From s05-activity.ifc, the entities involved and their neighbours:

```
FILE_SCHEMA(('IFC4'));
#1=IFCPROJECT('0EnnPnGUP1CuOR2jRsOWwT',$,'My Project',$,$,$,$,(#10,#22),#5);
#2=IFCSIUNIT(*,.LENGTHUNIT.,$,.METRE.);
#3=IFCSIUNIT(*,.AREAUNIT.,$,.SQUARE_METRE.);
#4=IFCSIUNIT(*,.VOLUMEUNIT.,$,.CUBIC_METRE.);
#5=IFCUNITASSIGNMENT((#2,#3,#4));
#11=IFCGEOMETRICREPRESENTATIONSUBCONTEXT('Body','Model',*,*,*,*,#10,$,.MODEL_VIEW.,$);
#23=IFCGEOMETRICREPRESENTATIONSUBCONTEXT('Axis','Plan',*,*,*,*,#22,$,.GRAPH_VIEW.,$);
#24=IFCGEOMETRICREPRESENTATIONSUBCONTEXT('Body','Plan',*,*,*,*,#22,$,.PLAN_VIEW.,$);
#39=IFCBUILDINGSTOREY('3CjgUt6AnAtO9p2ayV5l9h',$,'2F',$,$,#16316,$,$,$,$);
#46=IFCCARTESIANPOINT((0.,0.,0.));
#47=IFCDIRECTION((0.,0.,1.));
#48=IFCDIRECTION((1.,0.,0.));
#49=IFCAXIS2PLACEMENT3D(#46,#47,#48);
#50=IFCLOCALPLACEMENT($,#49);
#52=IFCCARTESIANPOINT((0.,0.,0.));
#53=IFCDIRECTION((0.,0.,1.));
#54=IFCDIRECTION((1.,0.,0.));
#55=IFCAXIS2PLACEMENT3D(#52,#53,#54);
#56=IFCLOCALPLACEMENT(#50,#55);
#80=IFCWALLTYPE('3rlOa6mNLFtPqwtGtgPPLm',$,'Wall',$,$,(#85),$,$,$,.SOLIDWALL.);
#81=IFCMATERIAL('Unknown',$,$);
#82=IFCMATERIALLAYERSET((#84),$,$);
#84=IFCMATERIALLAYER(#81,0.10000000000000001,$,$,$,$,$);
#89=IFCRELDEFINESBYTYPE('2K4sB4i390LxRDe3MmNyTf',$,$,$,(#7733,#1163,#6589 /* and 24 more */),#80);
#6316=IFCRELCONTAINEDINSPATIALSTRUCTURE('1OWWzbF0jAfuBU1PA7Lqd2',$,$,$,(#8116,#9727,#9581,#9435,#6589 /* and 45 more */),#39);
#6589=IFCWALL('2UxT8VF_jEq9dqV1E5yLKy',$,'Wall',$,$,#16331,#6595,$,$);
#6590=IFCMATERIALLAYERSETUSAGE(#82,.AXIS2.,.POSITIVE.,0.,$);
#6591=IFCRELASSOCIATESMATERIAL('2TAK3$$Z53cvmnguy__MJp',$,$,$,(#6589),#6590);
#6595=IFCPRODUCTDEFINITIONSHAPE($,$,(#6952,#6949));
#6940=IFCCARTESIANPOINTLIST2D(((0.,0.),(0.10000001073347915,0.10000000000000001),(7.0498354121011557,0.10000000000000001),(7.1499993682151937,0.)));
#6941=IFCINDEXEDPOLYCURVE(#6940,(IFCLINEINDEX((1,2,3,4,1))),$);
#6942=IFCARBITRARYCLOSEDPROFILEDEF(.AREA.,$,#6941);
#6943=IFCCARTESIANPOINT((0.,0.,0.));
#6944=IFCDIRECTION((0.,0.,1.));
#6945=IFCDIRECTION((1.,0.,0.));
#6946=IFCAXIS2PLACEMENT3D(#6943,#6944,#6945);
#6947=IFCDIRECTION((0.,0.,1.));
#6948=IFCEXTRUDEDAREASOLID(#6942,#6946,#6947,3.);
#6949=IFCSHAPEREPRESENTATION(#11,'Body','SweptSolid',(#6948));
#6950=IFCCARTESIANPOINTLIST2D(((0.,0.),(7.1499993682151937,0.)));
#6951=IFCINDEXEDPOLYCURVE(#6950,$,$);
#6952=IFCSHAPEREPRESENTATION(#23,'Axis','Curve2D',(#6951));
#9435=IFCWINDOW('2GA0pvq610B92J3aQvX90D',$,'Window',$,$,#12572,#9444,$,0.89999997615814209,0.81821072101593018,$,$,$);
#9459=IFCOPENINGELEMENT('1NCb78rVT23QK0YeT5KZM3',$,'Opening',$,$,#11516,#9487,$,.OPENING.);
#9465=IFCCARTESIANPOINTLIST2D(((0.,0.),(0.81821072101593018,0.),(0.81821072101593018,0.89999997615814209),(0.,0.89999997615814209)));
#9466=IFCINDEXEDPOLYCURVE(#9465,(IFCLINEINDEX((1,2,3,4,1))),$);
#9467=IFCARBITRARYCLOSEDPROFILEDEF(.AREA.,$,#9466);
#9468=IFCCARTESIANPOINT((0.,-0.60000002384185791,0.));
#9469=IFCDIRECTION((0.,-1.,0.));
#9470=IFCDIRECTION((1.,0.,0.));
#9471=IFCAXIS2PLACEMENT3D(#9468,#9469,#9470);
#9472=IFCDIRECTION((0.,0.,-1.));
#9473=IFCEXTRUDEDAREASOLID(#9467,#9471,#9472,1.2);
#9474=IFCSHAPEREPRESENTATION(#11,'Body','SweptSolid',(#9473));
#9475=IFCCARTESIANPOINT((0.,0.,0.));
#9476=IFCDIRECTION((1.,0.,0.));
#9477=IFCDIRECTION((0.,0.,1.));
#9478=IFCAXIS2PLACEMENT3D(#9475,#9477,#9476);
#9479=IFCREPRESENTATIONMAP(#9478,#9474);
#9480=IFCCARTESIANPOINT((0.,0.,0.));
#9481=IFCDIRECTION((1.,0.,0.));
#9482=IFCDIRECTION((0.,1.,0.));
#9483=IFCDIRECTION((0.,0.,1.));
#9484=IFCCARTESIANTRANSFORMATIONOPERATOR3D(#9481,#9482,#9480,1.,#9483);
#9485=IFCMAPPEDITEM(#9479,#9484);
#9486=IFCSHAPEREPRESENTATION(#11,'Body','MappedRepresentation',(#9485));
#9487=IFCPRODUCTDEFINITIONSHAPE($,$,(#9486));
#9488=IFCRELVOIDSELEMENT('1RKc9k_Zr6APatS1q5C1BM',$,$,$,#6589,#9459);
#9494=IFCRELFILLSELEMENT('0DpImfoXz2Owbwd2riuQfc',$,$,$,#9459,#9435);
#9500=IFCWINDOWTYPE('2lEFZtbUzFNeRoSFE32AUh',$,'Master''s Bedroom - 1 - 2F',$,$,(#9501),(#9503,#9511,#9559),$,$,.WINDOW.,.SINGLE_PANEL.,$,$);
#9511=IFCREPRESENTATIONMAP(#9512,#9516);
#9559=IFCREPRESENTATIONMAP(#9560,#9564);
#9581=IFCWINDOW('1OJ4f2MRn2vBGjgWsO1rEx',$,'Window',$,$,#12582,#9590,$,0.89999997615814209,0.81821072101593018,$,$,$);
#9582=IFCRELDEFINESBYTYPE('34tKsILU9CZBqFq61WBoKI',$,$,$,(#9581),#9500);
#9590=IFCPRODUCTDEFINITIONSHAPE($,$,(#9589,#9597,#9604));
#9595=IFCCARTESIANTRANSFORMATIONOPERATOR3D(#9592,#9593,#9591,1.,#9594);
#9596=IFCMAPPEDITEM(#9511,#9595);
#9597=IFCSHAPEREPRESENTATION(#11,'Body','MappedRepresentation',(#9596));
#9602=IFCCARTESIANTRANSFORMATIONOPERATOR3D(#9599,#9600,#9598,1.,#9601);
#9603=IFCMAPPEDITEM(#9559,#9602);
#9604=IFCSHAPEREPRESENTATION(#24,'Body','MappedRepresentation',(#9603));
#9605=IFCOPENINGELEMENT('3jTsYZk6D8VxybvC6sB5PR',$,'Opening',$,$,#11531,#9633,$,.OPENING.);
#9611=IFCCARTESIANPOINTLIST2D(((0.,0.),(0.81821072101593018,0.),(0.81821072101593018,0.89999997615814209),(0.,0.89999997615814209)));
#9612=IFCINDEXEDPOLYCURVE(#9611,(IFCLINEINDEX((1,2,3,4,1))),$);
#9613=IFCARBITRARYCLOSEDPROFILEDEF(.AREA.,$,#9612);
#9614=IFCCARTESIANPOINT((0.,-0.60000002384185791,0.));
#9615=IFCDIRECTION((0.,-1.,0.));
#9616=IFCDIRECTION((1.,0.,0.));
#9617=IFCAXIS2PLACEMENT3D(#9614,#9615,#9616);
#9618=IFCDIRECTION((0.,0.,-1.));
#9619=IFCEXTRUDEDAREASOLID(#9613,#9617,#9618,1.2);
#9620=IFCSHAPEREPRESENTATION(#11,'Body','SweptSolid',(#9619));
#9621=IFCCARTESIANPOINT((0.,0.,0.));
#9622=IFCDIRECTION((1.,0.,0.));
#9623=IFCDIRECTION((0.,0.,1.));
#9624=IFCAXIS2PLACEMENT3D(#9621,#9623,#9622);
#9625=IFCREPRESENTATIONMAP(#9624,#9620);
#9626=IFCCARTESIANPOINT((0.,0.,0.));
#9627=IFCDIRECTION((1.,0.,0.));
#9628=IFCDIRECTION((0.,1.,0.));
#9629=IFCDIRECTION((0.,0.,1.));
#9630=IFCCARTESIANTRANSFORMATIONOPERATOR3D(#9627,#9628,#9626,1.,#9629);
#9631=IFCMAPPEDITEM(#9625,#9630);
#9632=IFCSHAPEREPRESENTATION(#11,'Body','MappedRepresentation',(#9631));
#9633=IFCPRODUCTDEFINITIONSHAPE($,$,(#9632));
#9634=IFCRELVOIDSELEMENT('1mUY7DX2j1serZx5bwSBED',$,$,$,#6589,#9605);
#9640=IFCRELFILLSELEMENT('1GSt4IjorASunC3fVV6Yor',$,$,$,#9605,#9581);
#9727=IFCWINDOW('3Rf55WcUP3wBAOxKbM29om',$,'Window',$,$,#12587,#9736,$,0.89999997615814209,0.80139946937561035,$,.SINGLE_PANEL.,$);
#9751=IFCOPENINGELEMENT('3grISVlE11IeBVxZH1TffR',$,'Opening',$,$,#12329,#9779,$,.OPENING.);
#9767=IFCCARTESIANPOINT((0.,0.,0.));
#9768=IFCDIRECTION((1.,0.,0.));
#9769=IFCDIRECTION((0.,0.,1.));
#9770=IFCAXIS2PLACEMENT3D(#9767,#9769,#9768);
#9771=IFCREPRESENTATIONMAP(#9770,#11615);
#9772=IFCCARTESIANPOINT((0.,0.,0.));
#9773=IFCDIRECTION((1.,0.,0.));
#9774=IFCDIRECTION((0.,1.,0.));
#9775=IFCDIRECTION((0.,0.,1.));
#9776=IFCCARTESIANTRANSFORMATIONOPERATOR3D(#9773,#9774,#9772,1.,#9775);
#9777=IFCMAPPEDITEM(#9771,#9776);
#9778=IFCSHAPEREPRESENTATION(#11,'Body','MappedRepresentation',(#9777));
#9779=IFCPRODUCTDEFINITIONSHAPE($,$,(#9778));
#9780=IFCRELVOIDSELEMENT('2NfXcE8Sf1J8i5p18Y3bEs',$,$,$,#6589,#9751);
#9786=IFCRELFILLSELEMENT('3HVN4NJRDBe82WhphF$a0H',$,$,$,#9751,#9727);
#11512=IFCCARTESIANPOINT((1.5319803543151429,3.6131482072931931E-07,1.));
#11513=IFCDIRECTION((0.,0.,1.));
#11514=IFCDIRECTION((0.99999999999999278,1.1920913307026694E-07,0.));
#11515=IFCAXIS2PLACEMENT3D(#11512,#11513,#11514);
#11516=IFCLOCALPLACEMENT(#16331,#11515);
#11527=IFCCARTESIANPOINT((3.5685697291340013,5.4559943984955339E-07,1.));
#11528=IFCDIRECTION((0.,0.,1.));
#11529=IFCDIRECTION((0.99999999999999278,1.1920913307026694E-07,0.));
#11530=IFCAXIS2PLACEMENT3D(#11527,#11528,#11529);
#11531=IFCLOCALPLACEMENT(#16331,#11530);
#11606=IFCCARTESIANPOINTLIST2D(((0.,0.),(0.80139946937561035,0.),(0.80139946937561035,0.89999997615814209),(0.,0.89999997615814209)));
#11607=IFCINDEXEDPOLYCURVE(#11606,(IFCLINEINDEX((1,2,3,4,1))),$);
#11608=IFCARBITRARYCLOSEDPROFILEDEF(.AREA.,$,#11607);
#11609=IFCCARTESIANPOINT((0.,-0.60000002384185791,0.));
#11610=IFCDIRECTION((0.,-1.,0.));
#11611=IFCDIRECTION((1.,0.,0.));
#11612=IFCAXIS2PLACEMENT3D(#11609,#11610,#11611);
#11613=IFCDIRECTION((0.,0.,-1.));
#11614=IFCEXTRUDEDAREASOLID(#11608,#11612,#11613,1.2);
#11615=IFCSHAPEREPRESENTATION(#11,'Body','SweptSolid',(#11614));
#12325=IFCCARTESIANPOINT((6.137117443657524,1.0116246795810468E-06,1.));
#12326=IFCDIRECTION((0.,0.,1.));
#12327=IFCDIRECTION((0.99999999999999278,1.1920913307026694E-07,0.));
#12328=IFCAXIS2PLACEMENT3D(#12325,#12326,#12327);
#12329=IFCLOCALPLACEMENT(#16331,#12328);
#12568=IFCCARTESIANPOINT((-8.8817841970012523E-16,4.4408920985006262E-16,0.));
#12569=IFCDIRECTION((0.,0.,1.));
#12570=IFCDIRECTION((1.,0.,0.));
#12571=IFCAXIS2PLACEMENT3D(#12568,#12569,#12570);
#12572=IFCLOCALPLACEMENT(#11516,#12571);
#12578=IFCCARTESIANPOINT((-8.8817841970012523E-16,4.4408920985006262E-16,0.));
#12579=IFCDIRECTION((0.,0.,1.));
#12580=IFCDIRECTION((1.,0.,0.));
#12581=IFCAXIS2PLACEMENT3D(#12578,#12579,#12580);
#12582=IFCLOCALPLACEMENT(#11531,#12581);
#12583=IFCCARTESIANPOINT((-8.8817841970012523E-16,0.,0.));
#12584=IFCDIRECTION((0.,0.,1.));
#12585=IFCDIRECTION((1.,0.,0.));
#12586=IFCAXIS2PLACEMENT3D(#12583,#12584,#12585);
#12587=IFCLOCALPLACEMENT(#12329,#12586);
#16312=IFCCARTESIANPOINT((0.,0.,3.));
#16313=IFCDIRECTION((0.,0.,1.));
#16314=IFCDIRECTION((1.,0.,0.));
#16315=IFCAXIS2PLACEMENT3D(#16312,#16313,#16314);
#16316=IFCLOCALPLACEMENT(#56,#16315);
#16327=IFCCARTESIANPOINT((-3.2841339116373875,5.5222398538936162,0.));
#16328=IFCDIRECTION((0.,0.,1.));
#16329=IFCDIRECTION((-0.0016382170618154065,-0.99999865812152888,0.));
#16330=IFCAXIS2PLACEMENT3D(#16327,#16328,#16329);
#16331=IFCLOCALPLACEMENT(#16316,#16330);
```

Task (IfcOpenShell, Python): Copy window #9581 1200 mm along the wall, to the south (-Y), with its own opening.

```python
import ifcopenshell
import ifcopenshell.api.feature
import ifcopenshell.api.geometry
import ifcopenshell.api.root
import ifcopenshell.geom
import ifcopenshell.util.element
import ifcopenshell.util.placement
import ifcopenshell.util.shape

model = ifcopenshell.open("s05-activity.ifc")
settings = ifcopenshell.geom.settings()


def volume(element):
    """Net volume in cubic metres, openings subtracted."""
    shape = ifcopenshell.geom.create_shape(settings, element)
    return ifcopenshell.util.shape.get_volume(shape.geometry)


window = model.by_guid("1OJ4f2MRn2vBGjgWsO1rEx")
opening = window.FillsVoids[0].RelatingOpeningElement
wall = opening.VoidsElements[0].RelatingBuildingElement
before = volume(wall)
shift = ifcopenshell.util.placement.get_local_placement(wall.ObjectPlacement)[:3, 0] * 1.2

# copy_class copies the void relationship, type, container and properties, but no geometry.
new_opening = ifcopenshell.api.root.copy_class(model, product=opening)
new_opening.Representation = ifcopenshell.util.element.copy_deep(
    model, opening.Representation, exclude=["IfcGeometricRepresentationContext", "IfcRepresentationMap"]
)
new_window = ifcopenshell.api.root.copy_class(model, product=window)
new_window.Representation = ifcopenshell.util.element.copy_deep(
    model, window.Representation, exclude=["IfcGeometricRepresentationContext", "IfcRepresentationMap"]
)
ifcopenshell.api.feature.add_filling(model, opening=new_opening, element=new_window)

for old, new in ((opening, new_opening), (window, new_window)):
    matrix = ifcopenshell.util.placement.get_local_placement(old.ObjectPlacement)
    matrix[:3, 3] += shift
    ifcopenshell.api.geometry.edit_object_placement(model, product=new, matrix=matrix, is_si=False)

after = volume(wall)

print(f"wall volume {before:.3f} -> {after:.3f} m3")

model.write("s05-activity_v2.ifc")
```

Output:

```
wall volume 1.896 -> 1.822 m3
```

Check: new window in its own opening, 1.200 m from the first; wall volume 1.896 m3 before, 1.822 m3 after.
